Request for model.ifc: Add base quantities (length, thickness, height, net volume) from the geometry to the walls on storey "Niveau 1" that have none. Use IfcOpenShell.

First a look at what the model holds.

```python
import ifcopenshell
import ifcopenshell.util.element
import ifcopenshell.util.unit

model = ifcopenshell.open("model.ifc")
print(model.schema)
for unit_type in ("LENGTHUNIT", "AREAUNIT", "VOLUMEUNIT"):
    print(unit_type, ifcopenshell.util.unit.calculate_unit_scale(model, unit_type))
storey = next(s for s in model.by_type("IfcBuildingStorey") if s.Name == "Niveau 1")
walls = [e for e in ifcopenshell.util.element.get_decomposition(storey) if e.is_a("IfcWall")]
for e in sorted(walls, key=lambda e: e.id()):
    print(e.id(), e.is_a(), e.Name, list(ifcopenshell.util.element.get_psets(e, qtos_only=True)), sep=" | ")
```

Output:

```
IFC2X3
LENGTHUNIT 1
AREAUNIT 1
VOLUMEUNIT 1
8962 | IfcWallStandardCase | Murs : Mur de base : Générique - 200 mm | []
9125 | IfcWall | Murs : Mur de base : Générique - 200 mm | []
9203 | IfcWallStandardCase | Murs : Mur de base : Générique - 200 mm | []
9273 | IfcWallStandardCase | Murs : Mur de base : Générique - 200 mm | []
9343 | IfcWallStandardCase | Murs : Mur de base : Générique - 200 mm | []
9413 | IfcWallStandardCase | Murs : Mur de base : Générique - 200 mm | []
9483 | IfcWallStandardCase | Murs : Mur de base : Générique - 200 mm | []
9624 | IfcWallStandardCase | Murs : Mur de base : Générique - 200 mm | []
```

```python
import ifcopenshell
import ifcopenshell.api.pset
import ifcopenshell.geom
import ifcopenshell.util.element
import ifcopenshell.util.shape
import ifcopenshell.util.unit

model = ifcopenshell.open("model.ifc")
unit_scale = ifcopenshell.util.unit.calculate_unit_scale(model)
volume_scale = ifcopenshell.util.unit.calculate_unit_scale(model, "VOLUMEUNIT")
settings = ifcopenshell.geom.settings()

storey = next(s for s in model.by_type("IfcBuildingStorey") if s.Name == "Niveau 1")
walls = [e for e in ifcopenshell.util.element.get_decomposition(storey) if e.is_a("IfcWall")]

for e in sorted(walls, key=lambda e: e.id()):
    if ifcopenshell.util.element.get_psets(e, qtos_only=True, should_inherit=False):
        continue
    # Geometry comes back in metres, in the element's own axes.
    shape = ifcopenshell.geom.create_shape(settings, e)
    values = {
        "Length": ifcopenshell.util.shape.get_x(shape.geometry) / unit_scale,
        "Width": ifcopenshell.util.shape.get_y(shape.geometry) / unit_scale,
        "Height": ifcopenshell.util.shape.get_z(shape.geometry) / unit_scale,
        "NetVolume": ifcopenshell.util.shape.get_volume(shape.geometry) / volume_scale,
    }
    qto = ifcopenshell.api.pset.add_qto(model, product=e, name="BaseQuantities")
    ifcopenshell.api.pset.edit_qto(model, qto=qto, properties=values)
    print(e.id(), {k: round(v, 3) for k, v in values.items()})

model.write("model-out.ifc")
```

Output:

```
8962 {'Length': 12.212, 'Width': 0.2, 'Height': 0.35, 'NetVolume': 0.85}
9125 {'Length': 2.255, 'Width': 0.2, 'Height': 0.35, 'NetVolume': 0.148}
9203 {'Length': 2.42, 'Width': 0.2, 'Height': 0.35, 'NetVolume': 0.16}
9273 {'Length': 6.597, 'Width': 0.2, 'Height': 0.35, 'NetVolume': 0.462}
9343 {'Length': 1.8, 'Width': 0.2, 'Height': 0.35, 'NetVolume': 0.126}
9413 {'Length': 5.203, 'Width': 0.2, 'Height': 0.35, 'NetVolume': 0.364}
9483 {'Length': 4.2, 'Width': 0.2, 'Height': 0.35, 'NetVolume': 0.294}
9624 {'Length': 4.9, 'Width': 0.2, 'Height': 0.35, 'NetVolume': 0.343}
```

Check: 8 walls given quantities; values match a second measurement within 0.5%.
